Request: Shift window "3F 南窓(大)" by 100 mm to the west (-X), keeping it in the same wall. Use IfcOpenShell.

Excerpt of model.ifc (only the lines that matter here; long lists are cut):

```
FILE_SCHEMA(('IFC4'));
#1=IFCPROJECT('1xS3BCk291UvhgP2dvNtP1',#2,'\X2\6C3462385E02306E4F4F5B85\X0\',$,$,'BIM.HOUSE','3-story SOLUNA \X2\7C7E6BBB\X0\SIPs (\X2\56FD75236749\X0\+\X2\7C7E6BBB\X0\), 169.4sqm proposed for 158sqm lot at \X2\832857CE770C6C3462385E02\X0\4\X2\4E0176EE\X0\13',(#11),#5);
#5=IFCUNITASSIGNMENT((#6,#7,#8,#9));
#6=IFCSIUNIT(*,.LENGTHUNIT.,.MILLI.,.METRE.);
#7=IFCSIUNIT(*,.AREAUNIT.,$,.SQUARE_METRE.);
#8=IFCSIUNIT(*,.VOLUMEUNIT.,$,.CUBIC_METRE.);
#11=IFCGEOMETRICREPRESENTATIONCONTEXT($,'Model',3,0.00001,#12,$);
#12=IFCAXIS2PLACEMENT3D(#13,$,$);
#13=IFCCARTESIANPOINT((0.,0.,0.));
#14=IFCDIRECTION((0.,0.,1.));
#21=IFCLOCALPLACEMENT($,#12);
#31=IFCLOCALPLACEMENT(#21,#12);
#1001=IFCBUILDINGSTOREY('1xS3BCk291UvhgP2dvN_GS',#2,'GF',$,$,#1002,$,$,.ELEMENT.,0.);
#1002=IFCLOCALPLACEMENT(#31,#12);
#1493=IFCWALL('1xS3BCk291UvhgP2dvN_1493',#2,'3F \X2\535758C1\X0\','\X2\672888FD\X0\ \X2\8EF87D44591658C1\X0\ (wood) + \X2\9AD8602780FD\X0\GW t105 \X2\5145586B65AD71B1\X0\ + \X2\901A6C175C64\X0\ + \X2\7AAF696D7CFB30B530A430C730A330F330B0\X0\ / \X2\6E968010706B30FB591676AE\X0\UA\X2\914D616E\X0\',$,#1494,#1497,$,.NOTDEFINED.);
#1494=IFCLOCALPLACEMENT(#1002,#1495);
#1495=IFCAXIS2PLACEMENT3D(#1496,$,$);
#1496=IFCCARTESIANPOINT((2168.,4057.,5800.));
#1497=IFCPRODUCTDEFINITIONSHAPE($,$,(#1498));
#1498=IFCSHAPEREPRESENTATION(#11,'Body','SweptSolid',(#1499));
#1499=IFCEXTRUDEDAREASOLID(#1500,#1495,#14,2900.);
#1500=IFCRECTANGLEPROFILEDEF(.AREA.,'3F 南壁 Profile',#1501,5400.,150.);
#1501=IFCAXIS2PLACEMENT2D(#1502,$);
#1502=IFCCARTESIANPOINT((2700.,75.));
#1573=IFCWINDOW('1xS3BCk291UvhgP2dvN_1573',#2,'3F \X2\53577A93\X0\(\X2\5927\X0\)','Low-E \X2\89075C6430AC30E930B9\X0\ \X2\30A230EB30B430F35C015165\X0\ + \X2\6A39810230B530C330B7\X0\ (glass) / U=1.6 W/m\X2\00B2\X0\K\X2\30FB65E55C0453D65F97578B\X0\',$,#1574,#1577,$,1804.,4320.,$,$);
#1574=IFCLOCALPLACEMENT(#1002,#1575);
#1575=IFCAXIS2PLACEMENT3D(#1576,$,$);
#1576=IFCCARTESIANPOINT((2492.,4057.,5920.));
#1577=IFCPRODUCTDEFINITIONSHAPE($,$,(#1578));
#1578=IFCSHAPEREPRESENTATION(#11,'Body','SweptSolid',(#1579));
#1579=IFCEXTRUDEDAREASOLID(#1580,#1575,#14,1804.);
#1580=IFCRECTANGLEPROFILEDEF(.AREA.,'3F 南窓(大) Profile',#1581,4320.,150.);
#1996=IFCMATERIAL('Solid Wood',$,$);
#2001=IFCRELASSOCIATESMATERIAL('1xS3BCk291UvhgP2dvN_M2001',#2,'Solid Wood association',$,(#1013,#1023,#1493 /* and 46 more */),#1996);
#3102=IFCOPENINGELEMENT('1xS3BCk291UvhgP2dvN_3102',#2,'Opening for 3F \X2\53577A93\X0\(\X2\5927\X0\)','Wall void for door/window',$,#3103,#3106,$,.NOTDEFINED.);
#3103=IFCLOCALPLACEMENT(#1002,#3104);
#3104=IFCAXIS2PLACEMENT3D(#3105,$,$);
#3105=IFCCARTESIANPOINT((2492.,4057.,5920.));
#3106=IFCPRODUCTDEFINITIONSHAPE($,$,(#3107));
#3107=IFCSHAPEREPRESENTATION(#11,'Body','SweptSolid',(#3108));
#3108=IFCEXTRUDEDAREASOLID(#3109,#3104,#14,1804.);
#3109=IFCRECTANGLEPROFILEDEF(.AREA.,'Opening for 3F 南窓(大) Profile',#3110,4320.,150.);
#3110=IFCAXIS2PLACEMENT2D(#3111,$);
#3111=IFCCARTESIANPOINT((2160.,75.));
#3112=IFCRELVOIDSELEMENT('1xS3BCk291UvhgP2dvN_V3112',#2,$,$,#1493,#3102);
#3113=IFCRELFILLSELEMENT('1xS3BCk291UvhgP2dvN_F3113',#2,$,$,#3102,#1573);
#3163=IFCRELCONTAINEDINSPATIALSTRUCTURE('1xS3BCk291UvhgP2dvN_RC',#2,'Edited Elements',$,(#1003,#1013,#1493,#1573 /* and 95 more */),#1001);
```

```python
import ifcopenshell
import ifcopenshell.api.geometry
import ifcopenshell.util.placement

model = ifcopenshell.open("model.ifc")

window = model.by_guid("1xS3BCk291UvhgP2dvN_1573")
opening = window.FillsVoids[0].RelatingOpeningElement
wall = opening.VoidsElements[0].RelatingBuildingElement

wall_matrix = ifcopenshell.util.placement.get_local_placement(wall.ObjectPlacement)
shift = wall_matrix[:3, 0] * -100.0
before = ifcopenshell.util.placement.get_local_placement(window.ObjectPlacement)[:3, 3].copy()

# The window is not placed relative to its opening, so move both.
for product in (opening, window):
    matrix = ifcopenshell.util.placement.get_local_placement(product.ObjectPlacement)
    matrix[:3, 3] += shift
    ifcopenshell.api.geometry.edit_object_placement(model, product=product, matrix=matrix, is_si=False)

after = ifcopenshell.util.placement.get_local_placement(window.ObjectPlacement)[:3, 3]
print("window moved by", (after - before).round(3) + 0.0)

model.write("model_edited.ifc")
```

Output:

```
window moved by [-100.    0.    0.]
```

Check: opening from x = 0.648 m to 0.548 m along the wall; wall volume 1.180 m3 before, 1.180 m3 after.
